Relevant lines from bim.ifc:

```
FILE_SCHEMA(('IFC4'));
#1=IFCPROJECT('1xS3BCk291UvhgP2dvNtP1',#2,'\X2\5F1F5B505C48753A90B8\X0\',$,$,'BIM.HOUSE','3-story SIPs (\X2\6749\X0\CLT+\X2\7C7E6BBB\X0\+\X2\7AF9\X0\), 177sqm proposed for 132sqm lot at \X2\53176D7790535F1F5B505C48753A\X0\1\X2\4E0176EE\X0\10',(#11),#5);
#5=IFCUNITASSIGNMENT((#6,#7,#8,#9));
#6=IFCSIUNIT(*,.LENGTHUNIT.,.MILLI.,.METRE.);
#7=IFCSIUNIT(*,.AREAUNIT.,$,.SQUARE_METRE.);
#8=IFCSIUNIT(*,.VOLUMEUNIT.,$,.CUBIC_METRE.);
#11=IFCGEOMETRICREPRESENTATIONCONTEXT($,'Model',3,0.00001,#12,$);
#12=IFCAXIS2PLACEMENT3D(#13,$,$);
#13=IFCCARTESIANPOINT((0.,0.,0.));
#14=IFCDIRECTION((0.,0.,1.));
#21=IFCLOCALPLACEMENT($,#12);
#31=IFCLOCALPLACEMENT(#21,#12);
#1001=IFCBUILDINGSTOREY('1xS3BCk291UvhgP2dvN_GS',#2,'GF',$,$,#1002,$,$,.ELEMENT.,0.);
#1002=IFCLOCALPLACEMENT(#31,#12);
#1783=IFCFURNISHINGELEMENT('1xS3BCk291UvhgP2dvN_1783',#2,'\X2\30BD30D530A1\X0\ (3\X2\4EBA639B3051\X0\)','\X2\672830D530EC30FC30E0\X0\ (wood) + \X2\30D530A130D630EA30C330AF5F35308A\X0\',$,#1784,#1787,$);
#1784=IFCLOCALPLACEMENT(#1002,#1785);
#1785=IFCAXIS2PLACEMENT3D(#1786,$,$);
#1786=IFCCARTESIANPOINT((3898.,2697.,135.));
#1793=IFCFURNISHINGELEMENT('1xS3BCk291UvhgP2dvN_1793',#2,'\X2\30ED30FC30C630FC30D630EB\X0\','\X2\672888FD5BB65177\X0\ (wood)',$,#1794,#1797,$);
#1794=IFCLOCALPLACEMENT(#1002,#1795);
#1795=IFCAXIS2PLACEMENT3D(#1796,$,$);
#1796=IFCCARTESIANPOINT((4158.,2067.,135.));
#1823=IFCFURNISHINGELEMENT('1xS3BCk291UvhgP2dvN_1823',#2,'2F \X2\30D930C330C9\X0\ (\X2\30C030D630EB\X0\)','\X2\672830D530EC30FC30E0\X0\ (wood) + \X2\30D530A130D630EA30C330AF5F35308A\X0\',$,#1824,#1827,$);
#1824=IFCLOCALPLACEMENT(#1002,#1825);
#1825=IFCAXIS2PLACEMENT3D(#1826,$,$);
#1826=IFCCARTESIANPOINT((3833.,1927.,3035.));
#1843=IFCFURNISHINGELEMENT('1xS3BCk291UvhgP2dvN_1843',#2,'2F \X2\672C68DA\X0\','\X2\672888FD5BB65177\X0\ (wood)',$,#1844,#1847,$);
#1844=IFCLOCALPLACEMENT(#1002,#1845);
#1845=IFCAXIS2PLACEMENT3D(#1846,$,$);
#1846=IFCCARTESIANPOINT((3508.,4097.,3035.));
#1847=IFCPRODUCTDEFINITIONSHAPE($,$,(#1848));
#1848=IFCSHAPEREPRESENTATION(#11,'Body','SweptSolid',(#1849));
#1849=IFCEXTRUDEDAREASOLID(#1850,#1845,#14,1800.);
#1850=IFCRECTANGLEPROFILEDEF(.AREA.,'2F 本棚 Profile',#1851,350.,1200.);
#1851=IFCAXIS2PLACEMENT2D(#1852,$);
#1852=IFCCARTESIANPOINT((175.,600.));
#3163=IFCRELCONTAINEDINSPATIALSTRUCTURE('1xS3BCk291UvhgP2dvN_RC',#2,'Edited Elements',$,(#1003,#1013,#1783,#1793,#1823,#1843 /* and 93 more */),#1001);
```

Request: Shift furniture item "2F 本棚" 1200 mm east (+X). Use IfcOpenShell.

```python
import ifcopenshell
import ifcopenshell.api.geometry
import ifcopenshell.util.placement
import ifcopenshell.util.unit

model = ifcopenshell.open("bim.ifc")
unit_scale = ifcopenshell.util.unit.calculate_unit_scale(model)

item = model.by_id(1843)
matrix = ifcopenshell.util.placement.get_local_placement(item.ObjectPlacement)
matrix[0, 3] += 1.2 / unit_scale
ifcopenshell.api.geometry.edit_object_placement(model, product=item, matrix=matrix, is_si=False)

print(ifcopenshell.util.placement.get_local_placement(item.ObjectPlacement).round(3) + 0.0)

model.write("bim-out.ifc")
```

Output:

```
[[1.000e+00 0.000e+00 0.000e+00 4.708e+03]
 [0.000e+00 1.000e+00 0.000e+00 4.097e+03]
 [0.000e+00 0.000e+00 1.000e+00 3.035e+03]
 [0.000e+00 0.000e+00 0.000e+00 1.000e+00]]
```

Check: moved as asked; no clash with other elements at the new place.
